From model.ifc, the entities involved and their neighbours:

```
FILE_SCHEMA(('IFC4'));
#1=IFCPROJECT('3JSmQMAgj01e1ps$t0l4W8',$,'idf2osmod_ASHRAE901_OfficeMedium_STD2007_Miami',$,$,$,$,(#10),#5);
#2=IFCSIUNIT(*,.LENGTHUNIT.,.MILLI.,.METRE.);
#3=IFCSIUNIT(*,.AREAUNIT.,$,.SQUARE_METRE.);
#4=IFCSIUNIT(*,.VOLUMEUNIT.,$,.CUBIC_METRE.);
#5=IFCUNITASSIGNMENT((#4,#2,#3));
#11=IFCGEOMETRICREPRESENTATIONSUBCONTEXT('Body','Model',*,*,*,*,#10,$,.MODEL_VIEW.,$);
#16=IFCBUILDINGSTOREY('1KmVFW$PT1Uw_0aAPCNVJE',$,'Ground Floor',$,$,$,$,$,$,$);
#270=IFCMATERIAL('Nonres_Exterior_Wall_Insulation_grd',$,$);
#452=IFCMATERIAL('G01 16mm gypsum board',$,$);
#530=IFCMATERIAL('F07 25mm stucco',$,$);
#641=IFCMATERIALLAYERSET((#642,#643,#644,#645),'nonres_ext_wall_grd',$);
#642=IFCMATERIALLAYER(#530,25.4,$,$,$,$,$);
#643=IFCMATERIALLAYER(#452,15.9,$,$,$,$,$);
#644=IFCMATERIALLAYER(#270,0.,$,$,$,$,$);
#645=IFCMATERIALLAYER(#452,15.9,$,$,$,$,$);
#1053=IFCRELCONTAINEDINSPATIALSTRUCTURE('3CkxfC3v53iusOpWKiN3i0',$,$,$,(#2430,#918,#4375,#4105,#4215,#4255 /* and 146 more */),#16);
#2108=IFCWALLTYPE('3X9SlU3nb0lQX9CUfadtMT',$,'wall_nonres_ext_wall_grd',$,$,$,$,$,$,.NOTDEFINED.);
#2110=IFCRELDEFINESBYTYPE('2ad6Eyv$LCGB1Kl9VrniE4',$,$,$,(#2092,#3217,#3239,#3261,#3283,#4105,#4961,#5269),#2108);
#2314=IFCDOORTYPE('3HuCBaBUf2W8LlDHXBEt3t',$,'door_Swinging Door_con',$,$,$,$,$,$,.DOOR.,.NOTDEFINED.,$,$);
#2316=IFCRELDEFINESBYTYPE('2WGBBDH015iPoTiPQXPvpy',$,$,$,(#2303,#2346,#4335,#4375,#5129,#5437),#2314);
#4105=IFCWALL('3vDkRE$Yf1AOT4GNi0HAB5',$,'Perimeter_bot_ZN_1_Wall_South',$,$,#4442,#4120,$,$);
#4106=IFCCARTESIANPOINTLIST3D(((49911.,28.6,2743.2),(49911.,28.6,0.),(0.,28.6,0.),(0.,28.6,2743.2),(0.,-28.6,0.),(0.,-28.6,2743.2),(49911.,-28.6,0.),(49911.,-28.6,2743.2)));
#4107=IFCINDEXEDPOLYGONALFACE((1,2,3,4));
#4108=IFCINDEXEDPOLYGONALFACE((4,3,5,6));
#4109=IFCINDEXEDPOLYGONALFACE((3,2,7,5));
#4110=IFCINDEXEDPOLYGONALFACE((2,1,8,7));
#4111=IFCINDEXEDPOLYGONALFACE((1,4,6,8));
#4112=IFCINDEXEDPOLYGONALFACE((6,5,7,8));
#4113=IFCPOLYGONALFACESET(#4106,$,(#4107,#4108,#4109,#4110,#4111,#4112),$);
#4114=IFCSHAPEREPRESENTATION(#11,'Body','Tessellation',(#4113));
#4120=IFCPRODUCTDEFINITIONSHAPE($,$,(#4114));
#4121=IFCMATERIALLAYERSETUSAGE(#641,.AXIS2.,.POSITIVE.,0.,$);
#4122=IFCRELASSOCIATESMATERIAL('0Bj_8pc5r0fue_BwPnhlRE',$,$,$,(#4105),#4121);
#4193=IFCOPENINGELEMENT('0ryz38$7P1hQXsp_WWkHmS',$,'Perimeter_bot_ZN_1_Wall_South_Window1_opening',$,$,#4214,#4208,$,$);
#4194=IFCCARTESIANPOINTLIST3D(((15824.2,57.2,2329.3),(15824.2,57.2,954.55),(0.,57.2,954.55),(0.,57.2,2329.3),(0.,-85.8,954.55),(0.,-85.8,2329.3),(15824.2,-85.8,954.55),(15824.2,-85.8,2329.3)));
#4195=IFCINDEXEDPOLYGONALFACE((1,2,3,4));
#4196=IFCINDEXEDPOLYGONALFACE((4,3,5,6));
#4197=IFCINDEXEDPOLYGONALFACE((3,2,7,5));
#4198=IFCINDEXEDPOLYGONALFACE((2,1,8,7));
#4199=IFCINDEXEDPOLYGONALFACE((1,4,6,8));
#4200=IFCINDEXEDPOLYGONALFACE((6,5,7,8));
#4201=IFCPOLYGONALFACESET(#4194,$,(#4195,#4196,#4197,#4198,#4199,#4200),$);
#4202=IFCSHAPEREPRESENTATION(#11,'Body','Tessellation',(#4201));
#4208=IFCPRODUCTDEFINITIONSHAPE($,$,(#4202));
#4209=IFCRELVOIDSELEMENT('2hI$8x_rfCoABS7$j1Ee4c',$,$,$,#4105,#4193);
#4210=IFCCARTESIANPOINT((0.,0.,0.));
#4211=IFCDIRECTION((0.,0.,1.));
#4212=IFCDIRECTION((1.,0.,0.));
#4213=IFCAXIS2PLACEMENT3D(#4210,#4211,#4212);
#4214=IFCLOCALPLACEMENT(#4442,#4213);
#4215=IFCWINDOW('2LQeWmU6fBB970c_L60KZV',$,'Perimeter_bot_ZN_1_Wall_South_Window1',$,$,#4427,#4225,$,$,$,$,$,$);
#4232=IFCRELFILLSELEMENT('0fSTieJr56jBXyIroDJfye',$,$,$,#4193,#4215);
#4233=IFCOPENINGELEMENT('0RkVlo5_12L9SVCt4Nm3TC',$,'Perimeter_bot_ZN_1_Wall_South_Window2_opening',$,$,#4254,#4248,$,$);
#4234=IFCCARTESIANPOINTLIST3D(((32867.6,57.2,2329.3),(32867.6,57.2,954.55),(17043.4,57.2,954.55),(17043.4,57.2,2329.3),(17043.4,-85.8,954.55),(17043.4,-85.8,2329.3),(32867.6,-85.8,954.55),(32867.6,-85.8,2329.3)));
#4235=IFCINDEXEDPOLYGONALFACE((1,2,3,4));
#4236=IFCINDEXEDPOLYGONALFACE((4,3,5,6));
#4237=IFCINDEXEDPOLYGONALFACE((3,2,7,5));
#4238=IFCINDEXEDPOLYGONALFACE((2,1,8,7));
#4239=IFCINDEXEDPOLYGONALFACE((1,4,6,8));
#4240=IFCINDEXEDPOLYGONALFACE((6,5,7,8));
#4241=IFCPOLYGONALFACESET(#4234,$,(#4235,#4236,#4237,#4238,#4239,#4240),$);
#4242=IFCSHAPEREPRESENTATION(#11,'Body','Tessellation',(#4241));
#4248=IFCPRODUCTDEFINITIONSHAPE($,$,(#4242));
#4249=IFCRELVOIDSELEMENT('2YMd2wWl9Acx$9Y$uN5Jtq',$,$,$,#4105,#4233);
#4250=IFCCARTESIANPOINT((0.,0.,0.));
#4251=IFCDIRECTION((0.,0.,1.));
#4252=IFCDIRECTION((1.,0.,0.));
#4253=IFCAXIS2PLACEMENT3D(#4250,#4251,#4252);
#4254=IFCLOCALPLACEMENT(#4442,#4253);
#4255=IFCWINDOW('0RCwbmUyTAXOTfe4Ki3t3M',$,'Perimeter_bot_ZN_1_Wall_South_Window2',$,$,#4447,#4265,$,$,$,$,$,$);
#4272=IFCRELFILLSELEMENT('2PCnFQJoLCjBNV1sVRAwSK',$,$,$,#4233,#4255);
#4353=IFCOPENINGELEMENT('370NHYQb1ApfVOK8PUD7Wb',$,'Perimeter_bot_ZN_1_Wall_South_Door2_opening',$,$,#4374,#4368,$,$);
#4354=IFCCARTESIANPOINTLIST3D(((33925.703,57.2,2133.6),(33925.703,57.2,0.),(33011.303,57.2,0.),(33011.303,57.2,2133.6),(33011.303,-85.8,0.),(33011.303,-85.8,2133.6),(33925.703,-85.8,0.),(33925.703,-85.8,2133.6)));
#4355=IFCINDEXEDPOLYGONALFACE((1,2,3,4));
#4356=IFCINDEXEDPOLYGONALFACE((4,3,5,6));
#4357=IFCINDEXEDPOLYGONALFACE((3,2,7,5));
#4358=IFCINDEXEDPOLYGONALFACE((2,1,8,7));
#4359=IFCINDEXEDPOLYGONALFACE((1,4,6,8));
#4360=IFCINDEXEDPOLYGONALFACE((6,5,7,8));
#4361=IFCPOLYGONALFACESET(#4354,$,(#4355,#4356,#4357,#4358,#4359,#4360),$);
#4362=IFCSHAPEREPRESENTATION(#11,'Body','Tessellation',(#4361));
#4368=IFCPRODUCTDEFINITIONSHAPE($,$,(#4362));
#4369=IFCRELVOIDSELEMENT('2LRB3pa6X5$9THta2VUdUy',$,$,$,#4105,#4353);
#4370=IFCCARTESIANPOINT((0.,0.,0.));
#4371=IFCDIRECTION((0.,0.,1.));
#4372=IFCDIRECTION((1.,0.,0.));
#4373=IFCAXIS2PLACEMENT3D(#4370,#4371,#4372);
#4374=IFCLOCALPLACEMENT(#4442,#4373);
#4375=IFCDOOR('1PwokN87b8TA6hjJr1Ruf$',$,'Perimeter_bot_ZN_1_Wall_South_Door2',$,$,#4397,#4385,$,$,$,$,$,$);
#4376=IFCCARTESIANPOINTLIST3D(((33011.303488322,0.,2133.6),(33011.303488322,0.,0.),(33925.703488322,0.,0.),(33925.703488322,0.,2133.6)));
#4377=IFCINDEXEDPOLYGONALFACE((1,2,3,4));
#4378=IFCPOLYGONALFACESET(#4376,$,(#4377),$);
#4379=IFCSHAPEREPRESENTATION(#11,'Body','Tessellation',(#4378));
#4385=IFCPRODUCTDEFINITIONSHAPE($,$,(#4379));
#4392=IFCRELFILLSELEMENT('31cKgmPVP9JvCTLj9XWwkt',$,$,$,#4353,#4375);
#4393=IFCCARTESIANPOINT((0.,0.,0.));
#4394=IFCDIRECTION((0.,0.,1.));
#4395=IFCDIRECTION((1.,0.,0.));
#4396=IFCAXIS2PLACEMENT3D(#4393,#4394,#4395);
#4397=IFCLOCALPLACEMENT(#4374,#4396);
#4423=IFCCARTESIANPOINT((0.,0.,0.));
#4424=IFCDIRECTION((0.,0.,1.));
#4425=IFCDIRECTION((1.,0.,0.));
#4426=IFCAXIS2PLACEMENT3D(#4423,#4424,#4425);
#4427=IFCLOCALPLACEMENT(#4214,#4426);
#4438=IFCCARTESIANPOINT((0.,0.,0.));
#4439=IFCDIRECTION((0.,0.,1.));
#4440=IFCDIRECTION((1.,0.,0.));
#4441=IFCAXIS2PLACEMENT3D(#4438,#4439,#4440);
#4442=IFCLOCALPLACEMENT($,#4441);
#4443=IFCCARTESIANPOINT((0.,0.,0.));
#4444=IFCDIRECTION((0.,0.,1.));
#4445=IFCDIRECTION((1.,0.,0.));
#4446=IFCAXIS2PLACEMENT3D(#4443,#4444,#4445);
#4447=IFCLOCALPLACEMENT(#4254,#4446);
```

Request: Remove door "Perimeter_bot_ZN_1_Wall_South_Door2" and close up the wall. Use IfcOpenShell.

```python
import ifcopenshell
import ifcopenshell.api.feature
import ifcopenshell.api.root
import ifcopenshell.geom
import ifcopenshell.util.shape

model = ifcopenshell.open("model.ifc")
settings = ifcopenshell.geom.settings()


def volume(element):
    """Net volume in cubic metres, openings subtracted."""
    shape = ifcopenshell.geom.create_shape(settings, element)
    return ifcopenshell.util.shape.get_volume(shape.geometry)


door = model.by_guid("1PwokN87b8TA6hjJr1Ruf$")
opening = door.FillsVoids[0].RelatingOpeningElement
wall = opening.VoidsElements[0].RelatingBuildingElement
before = volume(wall)

ifcopenshell.api.root.remove_product(model, product=door)
ifcopenshell.api.feature.remove_feature(model, feature=opening)

after = volume(wall)

print(f"wall volume {before:.3f} -> {after:.3f} m3")

model.write("model_edited.ifc")
```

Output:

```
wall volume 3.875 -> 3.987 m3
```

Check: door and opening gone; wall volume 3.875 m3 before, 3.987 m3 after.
